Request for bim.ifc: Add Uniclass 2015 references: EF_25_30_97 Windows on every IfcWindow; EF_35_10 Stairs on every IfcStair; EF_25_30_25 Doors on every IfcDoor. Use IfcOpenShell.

First a look at what the model holds.

```python
import ifcopenshell

model = ifcopenshell.open("bim.ifc")
print(model.schema)
print("classifications:", [c.Name for c in model.by_type("IfcClassification")])
for ifc_class in ("IfcDoor", "IfcRoof", "IfcStair", "IfcWall", "IfcWindow"):
    print(ifc_class, len(model.by_type(ifc_class)))
```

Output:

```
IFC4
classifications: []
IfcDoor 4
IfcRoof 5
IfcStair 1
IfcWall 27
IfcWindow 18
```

```python
import ifcopenshell
import ifcopenshell.api.classification

model = ifcopenshell.open("bim.ifc")

system = ifcopenshell.api.classification.add_classification(model, classification="Uniclass 2015")

codes = {
    "IfcWindow": ("EF_25_30_97", "Windows"),
    "IfcStair": ("EF_35_10", "Stairs"),
    "IfcDoor": ("EF_25_30_25", "Doors"),
}
for ifc_class, (code, name) in codes.items():
    products = model.by_type(ifc_class)
    ifcopenshell.api.classification.add_reference(
        model, products=products, classification=system, identification=code, name=name
    )
    print(code, len(products))

model.write("bim_v2.ifc")
```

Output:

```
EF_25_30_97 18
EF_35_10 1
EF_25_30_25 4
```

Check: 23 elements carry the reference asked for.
